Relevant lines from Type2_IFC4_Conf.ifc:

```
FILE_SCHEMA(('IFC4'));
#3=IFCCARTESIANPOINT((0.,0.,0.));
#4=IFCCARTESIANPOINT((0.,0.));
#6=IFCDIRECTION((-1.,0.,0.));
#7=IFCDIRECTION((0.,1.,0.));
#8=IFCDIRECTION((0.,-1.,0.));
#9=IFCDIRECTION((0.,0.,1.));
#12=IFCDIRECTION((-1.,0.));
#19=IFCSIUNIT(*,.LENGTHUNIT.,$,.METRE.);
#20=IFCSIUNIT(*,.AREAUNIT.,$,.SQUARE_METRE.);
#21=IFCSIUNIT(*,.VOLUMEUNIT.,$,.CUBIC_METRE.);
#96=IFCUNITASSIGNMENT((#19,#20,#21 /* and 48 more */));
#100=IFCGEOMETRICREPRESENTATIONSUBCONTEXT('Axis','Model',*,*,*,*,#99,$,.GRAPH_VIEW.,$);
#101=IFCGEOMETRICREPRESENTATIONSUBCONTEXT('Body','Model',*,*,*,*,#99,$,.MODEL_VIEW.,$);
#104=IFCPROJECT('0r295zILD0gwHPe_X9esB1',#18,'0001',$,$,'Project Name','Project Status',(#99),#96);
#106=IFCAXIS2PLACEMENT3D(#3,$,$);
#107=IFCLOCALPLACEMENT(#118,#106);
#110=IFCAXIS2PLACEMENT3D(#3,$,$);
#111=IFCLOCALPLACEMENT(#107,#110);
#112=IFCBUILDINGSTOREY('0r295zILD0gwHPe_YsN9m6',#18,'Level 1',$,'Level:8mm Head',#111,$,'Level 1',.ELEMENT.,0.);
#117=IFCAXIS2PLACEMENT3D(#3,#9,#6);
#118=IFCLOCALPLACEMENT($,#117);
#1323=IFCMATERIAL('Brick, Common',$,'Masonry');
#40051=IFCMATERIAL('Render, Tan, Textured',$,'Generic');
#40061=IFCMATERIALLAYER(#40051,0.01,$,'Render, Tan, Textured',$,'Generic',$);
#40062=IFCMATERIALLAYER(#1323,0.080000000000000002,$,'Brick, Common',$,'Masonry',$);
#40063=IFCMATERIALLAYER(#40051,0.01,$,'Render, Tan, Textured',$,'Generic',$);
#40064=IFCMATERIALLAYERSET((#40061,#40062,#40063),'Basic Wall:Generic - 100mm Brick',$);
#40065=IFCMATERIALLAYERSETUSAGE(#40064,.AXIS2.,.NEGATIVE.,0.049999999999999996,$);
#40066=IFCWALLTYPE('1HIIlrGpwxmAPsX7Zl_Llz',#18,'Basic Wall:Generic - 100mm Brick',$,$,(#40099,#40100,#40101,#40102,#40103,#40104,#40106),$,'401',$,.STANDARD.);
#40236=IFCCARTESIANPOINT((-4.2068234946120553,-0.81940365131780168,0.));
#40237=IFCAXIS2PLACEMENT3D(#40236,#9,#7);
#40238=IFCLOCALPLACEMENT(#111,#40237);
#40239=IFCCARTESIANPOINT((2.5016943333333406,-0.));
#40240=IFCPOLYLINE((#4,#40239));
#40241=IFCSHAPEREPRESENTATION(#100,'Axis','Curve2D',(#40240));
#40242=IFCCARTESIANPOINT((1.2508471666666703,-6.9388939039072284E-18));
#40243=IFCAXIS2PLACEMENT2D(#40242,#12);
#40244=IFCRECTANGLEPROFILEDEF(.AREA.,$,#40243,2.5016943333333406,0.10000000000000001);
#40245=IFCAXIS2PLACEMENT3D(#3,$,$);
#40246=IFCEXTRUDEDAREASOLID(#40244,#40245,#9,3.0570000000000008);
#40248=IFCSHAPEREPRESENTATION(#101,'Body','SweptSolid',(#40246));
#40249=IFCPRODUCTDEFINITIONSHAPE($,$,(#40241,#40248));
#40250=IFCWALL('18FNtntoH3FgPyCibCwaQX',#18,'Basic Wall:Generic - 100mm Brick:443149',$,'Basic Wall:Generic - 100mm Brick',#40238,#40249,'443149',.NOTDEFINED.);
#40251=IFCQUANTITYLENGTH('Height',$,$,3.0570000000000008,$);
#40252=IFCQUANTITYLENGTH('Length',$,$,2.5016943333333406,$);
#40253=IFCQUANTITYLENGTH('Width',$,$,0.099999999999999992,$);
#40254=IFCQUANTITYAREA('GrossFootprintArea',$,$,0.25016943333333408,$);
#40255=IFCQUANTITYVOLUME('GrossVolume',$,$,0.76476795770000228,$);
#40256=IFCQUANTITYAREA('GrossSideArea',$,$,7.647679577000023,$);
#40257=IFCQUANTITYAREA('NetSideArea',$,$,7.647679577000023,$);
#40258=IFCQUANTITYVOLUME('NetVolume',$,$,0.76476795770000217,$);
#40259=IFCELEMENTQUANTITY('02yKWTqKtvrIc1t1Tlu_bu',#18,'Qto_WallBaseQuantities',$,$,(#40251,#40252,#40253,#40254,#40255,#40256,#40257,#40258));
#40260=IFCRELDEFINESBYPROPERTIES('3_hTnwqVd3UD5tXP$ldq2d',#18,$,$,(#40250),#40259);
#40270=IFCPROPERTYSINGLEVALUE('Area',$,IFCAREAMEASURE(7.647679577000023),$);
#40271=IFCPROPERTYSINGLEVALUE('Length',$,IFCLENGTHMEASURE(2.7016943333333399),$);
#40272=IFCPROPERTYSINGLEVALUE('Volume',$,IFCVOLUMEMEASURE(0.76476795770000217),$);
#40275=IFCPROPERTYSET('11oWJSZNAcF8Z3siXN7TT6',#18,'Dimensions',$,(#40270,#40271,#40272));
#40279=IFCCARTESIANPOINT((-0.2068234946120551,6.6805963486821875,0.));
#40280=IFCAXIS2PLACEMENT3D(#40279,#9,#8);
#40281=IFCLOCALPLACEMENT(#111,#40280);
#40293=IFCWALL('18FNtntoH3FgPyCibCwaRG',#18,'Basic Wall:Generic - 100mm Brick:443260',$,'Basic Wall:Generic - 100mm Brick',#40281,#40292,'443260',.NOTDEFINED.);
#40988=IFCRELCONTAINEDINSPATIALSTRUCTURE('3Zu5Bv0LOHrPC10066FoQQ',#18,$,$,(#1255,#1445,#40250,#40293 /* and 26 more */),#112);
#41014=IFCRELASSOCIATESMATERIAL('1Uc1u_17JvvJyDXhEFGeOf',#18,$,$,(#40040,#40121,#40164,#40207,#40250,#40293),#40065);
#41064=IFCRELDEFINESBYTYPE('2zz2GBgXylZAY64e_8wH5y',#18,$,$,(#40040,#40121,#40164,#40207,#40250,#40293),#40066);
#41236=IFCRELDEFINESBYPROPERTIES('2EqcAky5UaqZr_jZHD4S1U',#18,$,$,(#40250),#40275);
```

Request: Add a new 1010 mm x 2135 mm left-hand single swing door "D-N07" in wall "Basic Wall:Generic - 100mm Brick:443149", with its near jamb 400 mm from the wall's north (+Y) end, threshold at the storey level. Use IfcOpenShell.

```python
import numpy as np
import ifcopenshell
import ifcopenshell.api.feature
import ifcopenshell.api.geometry
import ifcopenshell.api.pset
import ifcopenshell.api.root
import ifcopenshell.api.spatial
import ifcopenshell.geom
import ifcopenshell.util.element
import ifcopenshell.util.placement
import ifcopenshell.util.representation
import ifcopenshell.util.shape
import ifcopenshell.util.unit

model = ifcopenshell.open("Type2_IFC4_Conf.ifc")
unit_scale = ifcopenshell.util.unit.calculate_unit_scale(model)
area_scale = ifcopenshell.util.unit.calculate_unit_scale(model, "AREAUNIT")
volume_scale = ifcopenshell.util.unit.calculate_unit_scale(model, "VOLUMEUNIT")
settings = ifcopenshell.geom.settings()


def volume(element):
    """Net volume in cubic metres, openings subtracted."""
    shape = ifcopenshell.geom.create_shape(settings, element)
    return ifcopenshell.util.shape.get_volume(shape.geometry)


wall = model.by_guid("18FNtntoH3FgPyCibCwaQX")
storey = ifcopenshell.util.element.get_container(wall, ifc_class="IfcBuildingStorey")
context = ifcopenshell.util.representation.get_context(model, "Model", "Body", "MODEL_VIEW")
before = volume(wall)

width, height, from_end, sill = 1.01, 2.135, 0.4, 0.0  # metres

# The wall runs along its own X axis, and the end named is its -X end.
wall_shape = ifcopenshell.geom.create_shape(settings, wall)
x, y, z = ifcopenshell.util.shape.get_vertices(wall_shape.geometry).T
start = x.min() + from_end
face, thickness = float(y.min()), float(y.max() - y.min())
wall_matrix = ifcopenshell.util.placement.get_local_placement(wall.ObjectPlacement)
level = ifcopenshell.util.placement.get_local_placement(storey.ObjectPlacement)[2, 3]


def in_wall(x, y):
    """Placement at x, y metres in the wall's axes, at sill height."""
    matrix = wall_matrix.copy()
    matrix[:, 3] = wall_matrix @ np.array([x / unit_scale, y / unit_scale, 0.0, 1.0])
    matrix[2, 3] = level + sill / unit_scale
    return matrix


# Opening: a box that overshoots both wall faces by 50 mm.
opening = ifcopenshell.api.root.create_entity(model, ifc_class="IfcOpeningElement", predefined_type="OPENING")
box = ifcopenshell.api.geometry.add_wall_representation(
    model, context=context, length=width, height=height, thickness=thickness + 0.1
)
ifcopenshell.api.geometry.assign_representation(model, product=opening, representation=box)
ifcopenshell.api.geometry.edit_object_placement(model, product=opening, matrix=in_wall(start, face - 0.05), is_si=False)
ifcopenshell.api.feature.add_feature(model, feature=opening, element=wall)

door = ifcopenshell.api.root.create_entity(model, ifc_class="IfcDoor", name="D-N07", predefined_type="DOOR")
door.OverallWidth, door.OverallHeight = width / unit_scale, height / unit_scale
door.OperationType = "SINGLE_SWING_LEFT"
body = ifcopenshell.api.geometry.add_door_representation(
    model,
    context=context,
    overall_width=door.OverallWidth,
    overall_height=door.OverallHeight,
    operation_type="SINGLE_SWING_LEFT",
    lining_properties={"LiningDepth": thickness / unit_scale, "ThresholdDepth": thickness / unit_scale},
)
ifcopenshell.api.geometry.assign_representation(model, product=door, representation=body)
ifcopenshell.api.spatial.assign_container(model, products=[door], relating_structure=storey)
ifcopenshell.api.feature.add_filling(model, opening=opening, element=door)

# The lining spans the wall, so the door starts at the wall face.
ifcopenshell.api.geometry.edit_object_placement(model, product=door, matrix=in_wall(start, face), is_si=False)

after = volume(wall)

# Update the wall's stored quantities.
qto = model.by_id(ifcopenshell.util.element.get_pset(wall, "Qto_WallBaseQuantities", should_inherit=False)["id"])
ifcopenshell.api.pset.edit_qto(model, qto=qto, properties={
    "NetSideArea": after / thickness / area_scale,
    "NetVolume": after / volume_scale,
})
pset = model.by_id(ifcopenshell.util.element.get_pset(wall, "Dimensions", should_inherit=False)["id"])
ifcopenshell.api.pset.edit_pset(model, pset=pset, properties={
    "Area": model.create_entity("IfcAreaMeasure", after / thickness / area_scale),
    "Volume": model.create_entity("IfcVolumeMeasure", after / volume_scale),
})

print(f"wall volume {before:.3f} -> {after:.3f} m3")

model.write("Type2_IFC4_Conf_v2.ifc")
```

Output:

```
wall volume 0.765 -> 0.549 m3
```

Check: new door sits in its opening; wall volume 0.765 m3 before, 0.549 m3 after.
